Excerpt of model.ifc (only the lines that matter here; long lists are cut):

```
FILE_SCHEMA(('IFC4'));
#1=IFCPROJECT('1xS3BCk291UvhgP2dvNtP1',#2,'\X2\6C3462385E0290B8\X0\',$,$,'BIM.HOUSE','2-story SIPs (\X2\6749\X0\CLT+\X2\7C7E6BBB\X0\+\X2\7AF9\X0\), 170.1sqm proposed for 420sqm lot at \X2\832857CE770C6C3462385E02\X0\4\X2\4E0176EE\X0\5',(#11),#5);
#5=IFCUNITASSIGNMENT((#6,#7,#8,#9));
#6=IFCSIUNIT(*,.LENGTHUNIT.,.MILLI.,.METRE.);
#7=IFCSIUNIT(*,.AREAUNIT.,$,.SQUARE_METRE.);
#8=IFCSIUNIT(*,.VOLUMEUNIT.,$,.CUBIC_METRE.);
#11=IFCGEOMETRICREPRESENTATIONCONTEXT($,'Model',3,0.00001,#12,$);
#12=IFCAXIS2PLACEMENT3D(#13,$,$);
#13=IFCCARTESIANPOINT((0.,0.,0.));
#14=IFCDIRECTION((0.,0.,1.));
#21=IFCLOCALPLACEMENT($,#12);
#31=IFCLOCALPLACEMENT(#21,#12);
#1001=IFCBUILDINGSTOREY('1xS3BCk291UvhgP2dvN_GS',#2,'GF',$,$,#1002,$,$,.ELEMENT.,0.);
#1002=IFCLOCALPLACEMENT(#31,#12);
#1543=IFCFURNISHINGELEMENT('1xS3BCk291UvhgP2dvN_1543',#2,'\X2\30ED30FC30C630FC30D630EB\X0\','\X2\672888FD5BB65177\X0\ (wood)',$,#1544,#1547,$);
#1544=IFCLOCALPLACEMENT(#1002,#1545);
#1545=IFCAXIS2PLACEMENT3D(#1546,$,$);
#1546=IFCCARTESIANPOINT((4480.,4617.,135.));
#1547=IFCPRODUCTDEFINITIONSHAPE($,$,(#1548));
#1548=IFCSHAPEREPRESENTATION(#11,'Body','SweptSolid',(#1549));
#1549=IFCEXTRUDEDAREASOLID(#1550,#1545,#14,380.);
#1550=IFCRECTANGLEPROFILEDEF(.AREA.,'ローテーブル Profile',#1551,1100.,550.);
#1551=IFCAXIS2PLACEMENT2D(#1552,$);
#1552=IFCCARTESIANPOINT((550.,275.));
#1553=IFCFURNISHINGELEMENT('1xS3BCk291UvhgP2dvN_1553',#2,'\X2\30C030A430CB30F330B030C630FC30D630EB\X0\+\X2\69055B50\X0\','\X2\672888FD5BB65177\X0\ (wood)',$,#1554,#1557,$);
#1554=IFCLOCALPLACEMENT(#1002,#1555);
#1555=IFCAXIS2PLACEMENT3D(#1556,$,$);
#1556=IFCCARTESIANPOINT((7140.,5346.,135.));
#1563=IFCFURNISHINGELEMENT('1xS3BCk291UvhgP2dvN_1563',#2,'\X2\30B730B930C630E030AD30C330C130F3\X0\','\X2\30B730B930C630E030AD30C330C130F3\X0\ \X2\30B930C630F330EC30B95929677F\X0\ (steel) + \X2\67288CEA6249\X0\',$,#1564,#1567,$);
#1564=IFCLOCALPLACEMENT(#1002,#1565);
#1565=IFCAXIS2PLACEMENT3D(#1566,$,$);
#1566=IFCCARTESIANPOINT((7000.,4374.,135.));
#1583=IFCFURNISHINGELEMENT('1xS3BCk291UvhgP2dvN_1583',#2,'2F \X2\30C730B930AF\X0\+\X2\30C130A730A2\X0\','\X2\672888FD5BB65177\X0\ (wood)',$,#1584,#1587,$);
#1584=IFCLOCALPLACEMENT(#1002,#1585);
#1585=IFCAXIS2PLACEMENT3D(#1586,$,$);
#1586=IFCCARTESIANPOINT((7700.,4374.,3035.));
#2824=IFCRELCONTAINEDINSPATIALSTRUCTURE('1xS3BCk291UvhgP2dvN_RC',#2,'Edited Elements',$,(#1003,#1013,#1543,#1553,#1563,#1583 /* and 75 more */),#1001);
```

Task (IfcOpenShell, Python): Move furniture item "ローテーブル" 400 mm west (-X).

```python
import ifcopenshell
import ifcopenshell.api.geometry
import ifcopenshell.util.placement

model = ifcopenshell.open("model.ifc")

item = model.by_guid("1xS3BCk291UvhgP2dvN_1543")
matrix = ifcopenshell.util.placement.get_local_placement(item.ObjectPlacement)
matrix[0, 3] -= 400.0
ifcopenshell.api.geometry.edit_object_placement(model, product=item, matrix=matrix, is_si=False)

print(ifcopenshell.util.placement.get_local_placement(item.ObjectPlacement).round(3) + 0.0)

model.write("model-out.ifc")
```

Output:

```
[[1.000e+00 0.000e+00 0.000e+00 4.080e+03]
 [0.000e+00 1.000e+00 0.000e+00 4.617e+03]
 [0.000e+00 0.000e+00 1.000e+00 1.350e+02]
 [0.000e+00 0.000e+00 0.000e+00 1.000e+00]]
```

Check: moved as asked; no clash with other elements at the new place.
